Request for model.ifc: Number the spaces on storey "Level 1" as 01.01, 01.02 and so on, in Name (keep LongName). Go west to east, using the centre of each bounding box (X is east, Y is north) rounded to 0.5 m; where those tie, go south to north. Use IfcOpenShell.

First a look at what the model holds.

```python
import ifcopenshell
import ifcopenshell.util.element
import ifcopenshell.util.placement

model = ifcopenshell.open("model.ifc")
print(model.schema)
storey = next(s for s in model.by_type("IfcBuildingStorey") if s.Name == "Level 1")
spaces = [e for e in ifcopenshell.util.element.get_decomposition(storey) if e.is_a("IfcSpace")]
for e in sorted(spaces, key=lambda e: e.id()):
    origin = ifcopenshell.util.placement.get_local_placement(e.ObjectPlacement)[:3, 3]
    print(e.id(), e.Name, e.LongName, origin.round(2) + 0.0, sep=" | ")
```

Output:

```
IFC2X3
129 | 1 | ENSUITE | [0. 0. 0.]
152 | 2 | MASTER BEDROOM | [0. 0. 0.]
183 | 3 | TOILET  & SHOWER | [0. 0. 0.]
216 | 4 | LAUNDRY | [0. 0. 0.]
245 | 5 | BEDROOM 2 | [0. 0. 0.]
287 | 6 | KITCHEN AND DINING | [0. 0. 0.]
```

```python
import ifcopenshell
import ifcopenshell.geom
import ifcopenshell.util.element
import ifcopenshell.util.shape

model = ifcopenshell.open("model.ifc")
settings = ifcopenshell.geom.settings()
settings.set("use-world-coords", True)


def centre(element):
    shape = ifcopenshell.geom.create_shape(settings, element)
    return ifcopenshell.util.shape.get_bbox_centroid(shape.geometry)


storey = next(s for s in model.by_type("IfcBuildingStorey") if s.Name == "Level 1")
spaces = [e for e in ifcopenshell.util.element.get_decomposition(storey) if e.is_a("IfcSpace")]

# Insertion points can sit at a corner or the storey origin, so sort by the geometry (in metres).
centres = {e: centre(e) for e in spaces}
spaces.sort(key=lambda e: (round(centres[e][0] / 0.5), centres[e][1]))

for i, e in enumerate(spaces, start=1):
    number = f"01.{i:02d}"
    e.Name = number
    print(e.id(), number)

model.write("model_v2.ifc")
```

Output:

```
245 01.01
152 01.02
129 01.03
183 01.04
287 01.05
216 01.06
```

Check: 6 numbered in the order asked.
